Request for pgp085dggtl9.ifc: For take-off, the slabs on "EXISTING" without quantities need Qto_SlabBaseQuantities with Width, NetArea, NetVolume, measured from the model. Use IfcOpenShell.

First a look at what the model holds.

```python
import ifcopenshell
import ifcopenshell.util.element
import ifcopenshell.util.unit

model = ifcopenshell.open("pgp085dggtl9.ifc")
print(model.schema)
for unit_type in ("LENGTHUNIT", "AREAUNIT", "VOLUMEUNIT"):
    print(unit_type, ifcopenshell.util.unit.calculate_unit_scale(model, unit_type))
storey = next(s for s in model.by_type("IfcBuildingStorey") if s.Name == "EXISTING")
slabs = [e for e in ifcopenshell.util.element.get_decomposition(storey) if e.is_a("IfcSlab")]
for e in sorted(slabs, key=lambda e: e.id()):
    print(e.id(), e.is_a(), e.Name, list(ifcopenshell.util.element.get_psets(e, qtos_only=True)), sep=" | ")
```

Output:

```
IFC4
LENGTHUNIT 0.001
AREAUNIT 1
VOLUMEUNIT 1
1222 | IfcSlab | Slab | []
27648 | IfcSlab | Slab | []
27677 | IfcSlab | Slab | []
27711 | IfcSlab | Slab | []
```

```python
import ifcopenshell
import ifcopenshell.api.pset
import ifcopenshell.geom
import ifcopenshell.util.element
import ifcopenshell.util.shape
import ifcopenshell.util.unit

model = ifcopenshell.open("pgp085dggtl9.ifc")
unit_scale = ifcopenshell.util.unit.calculate_unit_scale(model)
area_scale = ifcopenshell.util.unit.calculate_unit_scale(model, "AREAUNIT")
volume_scale = ifcopenshell.util.unit.calculate_unit_scale(model, "VOLUMEUNIT")
settings = ifcopenshell.geom.settings()

storey = next(s for s in model.by_type("IfcBuildingStorey") if s.Name == "EXISTING")
slabs = [e for e in ifcopenshell.util.element.get_decomposition(storey) if e.is_a("IfcSlab")]

for e in sorted(slabs, key=lambda e: e.id()):
    if ifcopenshell.util.element.get_psets(e, qtos_only=True, should_inherit=False):
        continue
    # Geometry comes back in metres, in the element's own axes.
    shape = ifcopenshell.geom.create_shape(settings, e)
    values = {
        "Width": ifcopenshell.util.shape.get_z(shape.geometry) / unit_scale,
        "NetArea": ifcopenshell.util.shape.get_footprint_area(shape.geometry) / area_scale,
        "NetVolume": ifcopenshell.util.shape.get_volume(shape.geometry) / volume_scale,
    }
    qto = ifcopenshell.api.pset.add_qto(model, product=e, name="Qto_SlabBaseQuantities")
    ifcopenshell.api.pset.edit_qto(model, qto=qto, properties=values)
    print(e.id(), {k: round(v, 3) for k, v in values.items()})

model.write("pgp085dggtl9_rev.ifc")
```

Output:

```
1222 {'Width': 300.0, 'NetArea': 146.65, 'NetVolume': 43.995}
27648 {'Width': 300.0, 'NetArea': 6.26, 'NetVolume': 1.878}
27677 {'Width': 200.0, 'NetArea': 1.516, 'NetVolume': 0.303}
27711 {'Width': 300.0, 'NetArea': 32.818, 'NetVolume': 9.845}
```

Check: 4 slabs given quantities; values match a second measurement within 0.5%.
